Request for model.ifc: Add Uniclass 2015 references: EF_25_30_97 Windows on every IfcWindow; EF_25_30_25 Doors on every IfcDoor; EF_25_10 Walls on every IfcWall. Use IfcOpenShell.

First a look at what the model holds.

```python
import ifcopenshell

model = ifcopenshell.open("model.ifc")
print(model.schema)
print("classifications:", [c.Name for c in model.by_type("IfcClassification")])
for ifc_class in ("IfcDoor", "IfcRoof", "IfcStair", "IfcWall", "IfcWindow"):
    print(ifc_class, len(model.by_type(ifc_class)))
```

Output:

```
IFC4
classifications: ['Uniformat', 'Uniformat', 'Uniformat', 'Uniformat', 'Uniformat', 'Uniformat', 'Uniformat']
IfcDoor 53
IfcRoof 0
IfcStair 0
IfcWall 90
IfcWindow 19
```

```python
import ifcopenshell
import ifcopenshell.api.classification

model = ifcopenshell.open("model.ifc")

system = ifcopenshell.api.classification.add_classification(model, classification="Uniclass 2015")

codes = {
    "IfcWindow": ("EF_25_30_97", "Windows"),
    "IfcDoor": ("EF_25_30_25", "Doors"),
    "IfcWall": ("EF_25_10", "Walls"),
}
for ifc_class, (code, name) in codes.items():
    products = model.by_type(ifc_class)
    ifcopenshell.api.classification.add_reference(
        model, products=products, classification=system, identification=code, name=name
    )
    print(code, len(products))

model.write("model_edited.ifc")
```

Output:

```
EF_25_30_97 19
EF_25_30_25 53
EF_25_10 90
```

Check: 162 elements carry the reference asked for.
